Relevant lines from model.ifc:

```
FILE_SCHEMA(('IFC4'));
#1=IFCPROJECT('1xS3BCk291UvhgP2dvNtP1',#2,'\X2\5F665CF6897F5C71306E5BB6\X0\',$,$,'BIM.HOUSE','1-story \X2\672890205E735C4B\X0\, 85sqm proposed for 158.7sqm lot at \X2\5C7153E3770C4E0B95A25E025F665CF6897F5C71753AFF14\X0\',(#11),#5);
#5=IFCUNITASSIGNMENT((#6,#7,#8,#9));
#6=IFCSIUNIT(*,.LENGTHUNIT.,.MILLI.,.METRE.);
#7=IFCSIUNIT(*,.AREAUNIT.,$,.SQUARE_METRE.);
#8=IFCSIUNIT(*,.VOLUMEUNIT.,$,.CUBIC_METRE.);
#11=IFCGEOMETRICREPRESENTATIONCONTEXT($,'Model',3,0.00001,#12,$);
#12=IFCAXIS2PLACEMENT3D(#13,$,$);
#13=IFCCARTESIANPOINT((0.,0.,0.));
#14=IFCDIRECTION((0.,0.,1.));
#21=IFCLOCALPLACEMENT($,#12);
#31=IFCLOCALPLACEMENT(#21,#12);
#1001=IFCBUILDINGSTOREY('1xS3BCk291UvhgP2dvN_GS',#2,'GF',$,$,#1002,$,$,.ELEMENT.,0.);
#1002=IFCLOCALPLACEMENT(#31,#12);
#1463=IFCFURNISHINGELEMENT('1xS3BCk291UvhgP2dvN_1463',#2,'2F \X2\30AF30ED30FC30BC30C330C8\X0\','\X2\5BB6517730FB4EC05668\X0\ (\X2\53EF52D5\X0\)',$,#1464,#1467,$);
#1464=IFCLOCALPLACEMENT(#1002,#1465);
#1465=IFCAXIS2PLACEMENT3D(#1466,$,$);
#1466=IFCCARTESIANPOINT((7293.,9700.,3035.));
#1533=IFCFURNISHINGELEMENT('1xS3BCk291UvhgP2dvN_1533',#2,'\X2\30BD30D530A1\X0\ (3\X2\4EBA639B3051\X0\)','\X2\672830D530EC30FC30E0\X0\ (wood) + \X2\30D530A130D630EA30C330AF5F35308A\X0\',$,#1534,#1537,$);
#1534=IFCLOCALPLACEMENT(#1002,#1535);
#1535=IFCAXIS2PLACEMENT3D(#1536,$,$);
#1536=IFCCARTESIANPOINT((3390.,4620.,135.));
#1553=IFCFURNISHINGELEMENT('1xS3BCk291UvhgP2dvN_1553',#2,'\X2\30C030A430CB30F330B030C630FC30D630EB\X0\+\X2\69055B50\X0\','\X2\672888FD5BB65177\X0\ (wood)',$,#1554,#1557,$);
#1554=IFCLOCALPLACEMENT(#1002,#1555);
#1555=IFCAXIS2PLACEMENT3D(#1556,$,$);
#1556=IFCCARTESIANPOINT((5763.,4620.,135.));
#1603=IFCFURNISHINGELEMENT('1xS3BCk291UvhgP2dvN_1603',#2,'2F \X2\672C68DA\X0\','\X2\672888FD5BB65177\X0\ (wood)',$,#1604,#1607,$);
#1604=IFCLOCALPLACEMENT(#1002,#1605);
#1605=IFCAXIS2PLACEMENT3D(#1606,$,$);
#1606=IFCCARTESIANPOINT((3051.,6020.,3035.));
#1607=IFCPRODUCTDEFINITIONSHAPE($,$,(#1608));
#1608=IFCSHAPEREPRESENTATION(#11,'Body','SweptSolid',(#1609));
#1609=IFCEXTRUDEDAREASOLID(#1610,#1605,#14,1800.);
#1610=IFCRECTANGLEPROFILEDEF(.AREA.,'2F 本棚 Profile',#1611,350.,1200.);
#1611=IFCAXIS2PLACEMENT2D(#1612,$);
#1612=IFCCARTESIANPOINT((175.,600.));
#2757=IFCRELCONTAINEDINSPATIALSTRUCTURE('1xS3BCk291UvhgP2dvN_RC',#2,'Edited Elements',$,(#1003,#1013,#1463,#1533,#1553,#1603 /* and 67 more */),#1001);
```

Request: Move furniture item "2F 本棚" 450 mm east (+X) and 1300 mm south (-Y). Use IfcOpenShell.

```python
import ifcopenshell
import ifcopenshell.api.geometry
import ifcopenshell.util.placement
import ifcopenshell.util.unit

model = ifcopenshell.open("model.ifc")
unit_scale = ifcopenshell.util.unit.calculate_unit_scale(model)

item = model.by_guid("1xS3BCk291UvhgP2dvN_1603")
matrix = ifcopenshell.util.placement.get_local_placement(item.ObjectPlacement)
matrix[0, 3] += 0.45 / unit_scale
matrix[1, 3] -= 1.3 / unit_scale
ifcopenshell.api.geometry.edit_object_placement(model, product=item, matrix=matrix, is_si=False)

print(ifcopenshell.util.placement.get_local_placement(item.ObjectPlacement).round(3) + 0.0)

model.write("model_edited.ifc")
```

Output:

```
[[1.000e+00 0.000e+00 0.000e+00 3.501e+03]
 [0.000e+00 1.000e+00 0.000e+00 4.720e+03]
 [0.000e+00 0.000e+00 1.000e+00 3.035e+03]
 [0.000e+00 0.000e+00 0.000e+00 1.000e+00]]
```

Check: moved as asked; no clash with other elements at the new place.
